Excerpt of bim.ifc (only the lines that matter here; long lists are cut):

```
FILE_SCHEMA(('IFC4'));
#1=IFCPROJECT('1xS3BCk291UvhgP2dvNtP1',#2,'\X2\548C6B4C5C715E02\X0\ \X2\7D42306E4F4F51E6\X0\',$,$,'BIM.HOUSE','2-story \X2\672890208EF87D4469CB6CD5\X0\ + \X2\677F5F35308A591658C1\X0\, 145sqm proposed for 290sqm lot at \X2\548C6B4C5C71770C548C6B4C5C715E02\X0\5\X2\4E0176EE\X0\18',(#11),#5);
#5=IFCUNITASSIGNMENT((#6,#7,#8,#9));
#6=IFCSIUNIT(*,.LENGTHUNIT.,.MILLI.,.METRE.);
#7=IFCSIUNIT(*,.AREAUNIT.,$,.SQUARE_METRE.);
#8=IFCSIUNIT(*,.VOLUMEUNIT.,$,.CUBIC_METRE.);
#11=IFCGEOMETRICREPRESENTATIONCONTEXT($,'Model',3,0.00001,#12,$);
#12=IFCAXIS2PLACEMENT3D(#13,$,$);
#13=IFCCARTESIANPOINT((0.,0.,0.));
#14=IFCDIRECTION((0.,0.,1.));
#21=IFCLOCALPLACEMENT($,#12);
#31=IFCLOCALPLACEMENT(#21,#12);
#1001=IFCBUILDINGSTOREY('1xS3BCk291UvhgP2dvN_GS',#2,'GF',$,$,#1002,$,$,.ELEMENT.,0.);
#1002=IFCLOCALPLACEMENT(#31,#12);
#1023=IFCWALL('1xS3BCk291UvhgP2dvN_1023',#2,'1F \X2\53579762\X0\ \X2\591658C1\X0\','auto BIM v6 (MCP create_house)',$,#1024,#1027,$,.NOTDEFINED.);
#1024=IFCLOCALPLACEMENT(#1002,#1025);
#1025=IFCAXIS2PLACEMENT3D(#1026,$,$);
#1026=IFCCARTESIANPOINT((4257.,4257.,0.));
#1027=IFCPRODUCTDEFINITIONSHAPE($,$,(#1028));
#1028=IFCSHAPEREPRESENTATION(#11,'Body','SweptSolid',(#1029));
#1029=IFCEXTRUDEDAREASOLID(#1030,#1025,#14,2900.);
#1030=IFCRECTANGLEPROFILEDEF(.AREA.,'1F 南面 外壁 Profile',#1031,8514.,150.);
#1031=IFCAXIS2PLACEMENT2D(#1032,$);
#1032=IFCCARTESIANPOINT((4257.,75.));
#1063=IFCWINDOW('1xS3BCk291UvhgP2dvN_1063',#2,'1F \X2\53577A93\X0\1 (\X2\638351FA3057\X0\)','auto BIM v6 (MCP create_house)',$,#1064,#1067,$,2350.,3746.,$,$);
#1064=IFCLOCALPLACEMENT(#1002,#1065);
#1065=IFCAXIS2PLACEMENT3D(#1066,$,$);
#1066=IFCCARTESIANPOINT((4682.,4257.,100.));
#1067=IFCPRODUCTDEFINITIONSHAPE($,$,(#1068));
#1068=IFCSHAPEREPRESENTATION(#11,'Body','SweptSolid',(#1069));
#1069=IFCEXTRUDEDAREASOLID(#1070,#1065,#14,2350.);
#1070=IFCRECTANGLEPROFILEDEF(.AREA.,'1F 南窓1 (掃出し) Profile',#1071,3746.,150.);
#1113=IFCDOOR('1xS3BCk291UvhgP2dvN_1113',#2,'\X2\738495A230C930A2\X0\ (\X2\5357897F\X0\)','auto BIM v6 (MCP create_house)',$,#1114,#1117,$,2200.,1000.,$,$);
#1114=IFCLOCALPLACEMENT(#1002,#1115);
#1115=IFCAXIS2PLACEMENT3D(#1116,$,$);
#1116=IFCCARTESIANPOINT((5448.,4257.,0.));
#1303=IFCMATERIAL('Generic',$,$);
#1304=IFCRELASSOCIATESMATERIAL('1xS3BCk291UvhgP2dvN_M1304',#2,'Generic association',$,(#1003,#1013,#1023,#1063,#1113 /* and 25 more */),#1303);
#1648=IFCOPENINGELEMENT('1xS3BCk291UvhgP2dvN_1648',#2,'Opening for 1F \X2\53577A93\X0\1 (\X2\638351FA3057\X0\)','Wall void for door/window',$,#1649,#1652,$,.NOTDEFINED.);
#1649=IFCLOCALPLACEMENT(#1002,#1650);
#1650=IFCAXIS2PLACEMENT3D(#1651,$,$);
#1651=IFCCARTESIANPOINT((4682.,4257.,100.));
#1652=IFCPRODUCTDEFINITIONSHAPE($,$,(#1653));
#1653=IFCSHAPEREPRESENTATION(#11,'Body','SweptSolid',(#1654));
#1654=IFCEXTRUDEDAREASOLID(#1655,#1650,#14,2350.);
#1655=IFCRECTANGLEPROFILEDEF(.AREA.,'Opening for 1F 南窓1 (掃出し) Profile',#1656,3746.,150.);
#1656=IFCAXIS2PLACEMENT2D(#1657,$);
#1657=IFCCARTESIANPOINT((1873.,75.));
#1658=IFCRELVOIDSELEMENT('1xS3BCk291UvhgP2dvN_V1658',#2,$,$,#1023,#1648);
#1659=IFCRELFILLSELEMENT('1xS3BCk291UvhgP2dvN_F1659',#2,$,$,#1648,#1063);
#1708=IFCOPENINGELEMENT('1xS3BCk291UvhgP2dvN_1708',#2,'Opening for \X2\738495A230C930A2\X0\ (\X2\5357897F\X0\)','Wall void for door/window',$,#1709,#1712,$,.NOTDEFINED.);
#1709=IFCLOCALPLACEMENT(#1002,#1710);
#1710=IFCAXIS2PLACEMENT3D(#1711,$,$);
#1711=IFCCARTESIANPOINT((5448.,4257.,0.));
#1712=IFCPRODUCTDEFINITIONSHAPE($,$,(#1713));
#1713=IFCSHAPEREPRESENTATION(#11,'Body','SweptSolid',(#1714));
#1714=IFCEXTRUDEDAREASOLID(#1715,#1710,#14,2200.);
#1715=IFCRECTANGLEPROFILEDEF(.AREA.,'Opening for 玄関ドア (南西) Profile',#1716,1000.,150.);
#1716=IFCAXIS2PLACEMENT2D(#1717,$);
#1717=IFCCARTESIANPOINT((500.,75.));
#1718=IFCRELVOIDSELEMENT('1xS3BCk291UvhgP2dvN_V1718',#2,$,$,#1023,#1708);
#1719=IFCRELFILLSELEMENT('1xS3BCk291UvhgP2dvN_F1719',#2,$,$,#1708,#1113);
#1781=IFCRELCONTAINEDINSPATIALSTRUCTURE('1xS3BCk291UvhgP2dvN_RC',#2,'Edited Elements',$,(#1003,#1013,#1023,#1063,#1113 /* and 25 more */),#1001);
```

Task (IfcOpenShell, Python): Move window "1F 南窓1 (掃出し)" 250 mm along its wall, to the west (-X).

```python
import ifcopenshell
import ifcopenshell.api.geometry
import ifcopenshell.util.placement
import ifcopenshell.util.unit

model = ifcopenshell.open("bim.ifc")
unit_scale = ifcopenshell.util.unit.calculate_unit_scale(model)

window = model.by_guid("1xS3BCk291UvhgP2dvN_1063")
opening = window.FillsVoids[0].RelatingOpeningElement
wall = opening.VoidsElements[0].RelatingBuildingElement

wall_matrix = ifcopenshell.util.placement.get_local_placement(wall.ObjectPlacement)
shift = wall_matrix[:3, 0] * -0.25 / unit_scale
before = ifcopenshell.util.placement.get_local_placement(window.ObjectPlacement)[:3, 3].copy()

# The window is not placed relative to its opening, so move both.
for product in (opening, window):
    matrix = ifcopenshell.util.placement.get_local_placement(product.ObjectPlacement)
    matrix[:3, 3] += shift
    ifcopenshell.api.geometry.edit_object_placement(model, product=product, matrix=matrix, is_si=False)

after = ifcopenshell.util.placement.get_local_placement(window.ObjectPlacement)[:3, 3]
print("window moved by", (after - before).round(3) + 0.0)

model.write("bim_updated.ifc")
```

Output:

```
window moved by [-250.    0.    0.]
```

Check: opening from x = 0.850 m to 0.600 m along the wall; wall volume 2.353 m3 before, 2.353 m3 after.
